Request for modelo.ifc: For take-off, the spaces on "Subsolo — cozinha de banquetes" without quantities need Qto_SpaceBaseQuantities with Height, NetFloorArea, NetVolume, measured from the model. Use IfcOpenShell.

First a look at what the model holds.

```python
import ifcopenshell
import ifcopenshell.util.element
import ifcopenshell.util.unit

model = ifcopenshell.open("modelo.ifc")
print(model.schema)
for unit_type in ("LENGTHUNIT", "AREAUNIT", "VOLUMEUNIT"):
    print(unit_type, ifcopenshell.util.unit.calculate_unit_scale(model, unit_type))
storey = next(s for s in model.by_type("IfcBuildingStorey") if s.Name == "Subsolo — cozinha de banquetes")
spaces = [e for e in ifcopenshell.util.element.get_decomposition(storey) if e.is_a("IfcSpace")]
for e in sorted(spaces, key=lambda e: e.id()):
    print(e.id(), e.is_a(), e.Name, list(ifcopenshell.util.element.get_psets(e, qtos_only=True)), sep=" | ")
```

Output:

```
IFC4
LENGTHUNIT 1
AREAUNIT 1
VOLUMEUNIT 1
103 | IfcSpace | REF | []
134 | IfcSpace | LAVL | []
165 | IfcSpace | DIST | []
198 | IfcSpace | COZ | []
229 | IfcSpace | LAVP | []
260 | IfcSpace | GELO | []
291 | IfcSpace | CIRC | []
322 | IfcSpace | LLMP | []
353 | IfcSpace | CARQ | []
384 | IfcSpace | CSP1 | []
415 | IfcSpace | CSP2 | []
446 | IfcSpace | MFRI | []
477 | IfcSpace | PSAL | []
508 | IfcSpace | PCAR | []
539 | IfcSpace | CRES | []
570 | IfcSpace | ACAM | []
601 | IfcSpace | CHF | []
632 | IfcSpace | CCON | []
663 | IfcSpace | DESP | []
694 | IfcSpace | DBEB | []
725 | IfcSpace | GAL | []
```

```python
import ifcopenshell
import ifcopenshell.api.pset
import ifcopenshell.geom
import ifcopenshell.util.element
import ifcopenshell.util.shape
import ifcopenshell.util.unit

model = ifcopenshell.open("modelo.ifc")
unit_scale = ifcopenshell.util.unit.calculate_unit_scale(model)
area_scale = ifcopenshell.util.unit.calculate_unit_scale(model, "AREAUNIT")
volume_scale = ifcopenshell.util.unit.calculate_unit_scale(model, "VOLUMEUNIT")
settings = ifcopenshell.geom.settings()

storey = next(s for s in model.by_type("IfcBuildingStorey") if s.Name == "Subsolo — cozinha de banquetes")
spaces = [e for e in ifcopenshell.util.element.get_decomposition(storey) if e.is_a("IfcSpace")]

for e in sorted(spaces, key=lambda e: e.id()):
    if ifcopenshell.util.element.get_psets(e, qtos_only=True, should_inherit=False):
        continue
    # Geometry comes back in metres, in the element's own axes.
    shape = ifcopenshell.geom.create_shape(settings, e)
    values = {
        "Height": ifcopenshell.util.shape.get_z(shape.geometry) / unit_scale,
        "NetFloorArea": ifcopenshell.util.shape.get_footprint_area(shape.geometry) / area_scale,
        "NetVolume": ifcopenshell.util.shape.get_volume(shape.geometry) / volume_scale,
    }
    qto = ifcopenshell.api.pset.add_qto(model, product=e, name="Qto_SpaceBaseQuantities")
    ifcopenshell.api.pset.edit_qto(model, qto=qto, properties=values)
    print(e.id(), {k: round(v, 3) for k, v in values.items()})

model.write("modelo_v2.ifc")
```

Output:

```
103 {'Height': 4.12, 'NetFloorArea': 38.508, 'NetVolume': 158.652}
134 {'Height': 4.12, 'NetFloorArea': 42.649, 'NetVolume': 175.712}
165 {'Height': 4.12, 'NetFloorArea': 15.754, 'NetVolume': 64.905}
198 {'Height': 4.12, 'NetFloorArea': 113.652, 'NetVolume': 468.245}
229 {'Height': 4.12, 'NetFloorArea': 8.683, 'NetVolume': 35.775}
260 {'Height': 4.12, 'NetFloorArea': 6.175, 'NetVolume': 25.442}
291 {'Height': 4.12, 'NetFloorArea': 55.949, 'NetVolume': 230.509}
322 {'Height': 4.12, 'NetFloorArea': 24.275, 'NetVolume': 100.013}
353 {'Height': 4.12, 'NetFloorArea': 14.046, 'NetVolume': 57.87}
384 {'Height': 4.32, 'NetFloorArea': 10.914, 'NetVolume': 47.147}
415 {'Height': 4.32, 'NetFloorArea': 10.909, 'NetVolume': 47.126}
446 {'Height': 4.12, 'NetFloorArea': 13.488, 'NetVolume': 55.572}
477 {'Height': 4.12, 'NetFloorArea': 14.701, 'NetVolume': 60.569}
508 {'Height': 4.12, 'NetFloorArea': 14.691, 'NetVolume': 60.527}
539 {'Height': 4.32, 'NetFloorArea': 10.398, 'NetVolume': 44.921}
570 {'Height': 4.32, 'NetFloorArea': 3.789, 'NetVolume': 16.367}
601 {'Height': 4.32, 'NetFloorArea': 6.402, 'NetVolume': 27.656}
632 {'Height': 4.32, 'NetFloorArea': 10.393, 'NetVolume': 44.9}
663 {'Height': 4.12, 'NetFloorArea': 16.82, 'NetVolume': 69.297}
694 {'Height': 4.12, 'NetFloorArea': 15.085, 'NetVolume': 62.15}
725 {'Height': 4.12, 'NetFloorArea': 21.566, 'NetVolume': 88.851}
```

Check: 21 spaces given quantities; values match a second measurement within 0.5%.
